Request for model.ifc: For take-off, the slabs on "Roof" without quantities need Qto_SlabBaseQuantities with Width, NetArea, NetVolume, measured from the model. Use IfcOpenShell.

First a look at what the model holds.

```python
import ifcopenshell
import ifcopenshell.util.element
import ifcopenshell.util.unit

model = ifcopenshell.open("model.ifc")
print(model.schema)
for unit_type in ("LENGTHUNIT", "AREAUNIT", "VOLUMEUNIT"):
    print(unit_type, ifcopenshell.util.unit.calculate_unit_scale(model, unit_type))
storey = next(s for s in model.by_type("IfcBuildingStorey") if s.Name == "Roof")
slabs = [e for e in ifcopenshell.util.element.get_decomposition(storey) if e.is_a("IfcSlab")]
for e in sorted(slabs, key=lambda e: e.id()):
    print(e.id(), e.is_a(), e.Name, list(ifcopenshell.util.element.get_psets(e, qtos_only=True)), sep=" | ")
```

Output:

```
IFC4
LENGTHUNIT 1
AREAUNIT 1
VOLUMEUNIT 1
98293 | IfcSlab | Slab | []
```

```python
import ifcopenshell
import ifcopenshell.api.pset
import ifcopenshell.geom
import ifcopenshell.util.element
import ifcopenshell.util.shape
import ifcopenshell.util.unit

model = ifcopenshell.open("model.ifc")
unit_scale = ifcopenshell.util.unit.calculate_unit_scale(model)
area_scale = ifcopenshell.util.unit.calculate_unit_scale(model, "AREAUNIT")
volume_scale = ifcopenshell.util.unit.calculate_unit_scale(model, "VOLUMEUNIT")
settings = ifcopenshell.geom.settings()

storey = next(s for s in model.by_type("IfcBuildingStorey") if s.Name == "Roof")
slabs = [e for e in ifcopenshell.util.element.get_decomposition(storey) if e.is_a("IfcSlab")]

for e in sorted(slabs, key=lambda e: e.id()):
    if ifcopenshell.util.element.get_psets(e, qtos_only=True, should_inherit=False):
        continue
    # Geometry comes back in metres, in the element's own axes.
    shape = ifcopenshell.geom.create_shape(settings, e)
    values = {
        "Width": ifcopenshell.util.shape.get_z(shape.geometry) / unit_scale,
        "NetArea": ifcopenshell.util.shape.get_footprint_area(shape.geometry) / area_scale,
        "NetVolume": ifcopenshell.util.shape.get_volume(shape.geometry) / volume_scale,
    }
    qto = ifcopenshell.api.pset.add_qto(model, product=e, name="Qto_SlabBaseQuantities")
    ifcopenshell.api.pset.edit_qto(model, qto=qto, properties=values)
    print(e.id(), {k: round(v, 3) for k, v in values.items()})

model.write("model-out.ifc")
```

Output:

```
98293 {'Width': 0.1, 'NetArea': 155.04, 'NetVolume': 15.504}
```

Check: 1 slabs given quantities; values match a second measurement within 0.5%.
